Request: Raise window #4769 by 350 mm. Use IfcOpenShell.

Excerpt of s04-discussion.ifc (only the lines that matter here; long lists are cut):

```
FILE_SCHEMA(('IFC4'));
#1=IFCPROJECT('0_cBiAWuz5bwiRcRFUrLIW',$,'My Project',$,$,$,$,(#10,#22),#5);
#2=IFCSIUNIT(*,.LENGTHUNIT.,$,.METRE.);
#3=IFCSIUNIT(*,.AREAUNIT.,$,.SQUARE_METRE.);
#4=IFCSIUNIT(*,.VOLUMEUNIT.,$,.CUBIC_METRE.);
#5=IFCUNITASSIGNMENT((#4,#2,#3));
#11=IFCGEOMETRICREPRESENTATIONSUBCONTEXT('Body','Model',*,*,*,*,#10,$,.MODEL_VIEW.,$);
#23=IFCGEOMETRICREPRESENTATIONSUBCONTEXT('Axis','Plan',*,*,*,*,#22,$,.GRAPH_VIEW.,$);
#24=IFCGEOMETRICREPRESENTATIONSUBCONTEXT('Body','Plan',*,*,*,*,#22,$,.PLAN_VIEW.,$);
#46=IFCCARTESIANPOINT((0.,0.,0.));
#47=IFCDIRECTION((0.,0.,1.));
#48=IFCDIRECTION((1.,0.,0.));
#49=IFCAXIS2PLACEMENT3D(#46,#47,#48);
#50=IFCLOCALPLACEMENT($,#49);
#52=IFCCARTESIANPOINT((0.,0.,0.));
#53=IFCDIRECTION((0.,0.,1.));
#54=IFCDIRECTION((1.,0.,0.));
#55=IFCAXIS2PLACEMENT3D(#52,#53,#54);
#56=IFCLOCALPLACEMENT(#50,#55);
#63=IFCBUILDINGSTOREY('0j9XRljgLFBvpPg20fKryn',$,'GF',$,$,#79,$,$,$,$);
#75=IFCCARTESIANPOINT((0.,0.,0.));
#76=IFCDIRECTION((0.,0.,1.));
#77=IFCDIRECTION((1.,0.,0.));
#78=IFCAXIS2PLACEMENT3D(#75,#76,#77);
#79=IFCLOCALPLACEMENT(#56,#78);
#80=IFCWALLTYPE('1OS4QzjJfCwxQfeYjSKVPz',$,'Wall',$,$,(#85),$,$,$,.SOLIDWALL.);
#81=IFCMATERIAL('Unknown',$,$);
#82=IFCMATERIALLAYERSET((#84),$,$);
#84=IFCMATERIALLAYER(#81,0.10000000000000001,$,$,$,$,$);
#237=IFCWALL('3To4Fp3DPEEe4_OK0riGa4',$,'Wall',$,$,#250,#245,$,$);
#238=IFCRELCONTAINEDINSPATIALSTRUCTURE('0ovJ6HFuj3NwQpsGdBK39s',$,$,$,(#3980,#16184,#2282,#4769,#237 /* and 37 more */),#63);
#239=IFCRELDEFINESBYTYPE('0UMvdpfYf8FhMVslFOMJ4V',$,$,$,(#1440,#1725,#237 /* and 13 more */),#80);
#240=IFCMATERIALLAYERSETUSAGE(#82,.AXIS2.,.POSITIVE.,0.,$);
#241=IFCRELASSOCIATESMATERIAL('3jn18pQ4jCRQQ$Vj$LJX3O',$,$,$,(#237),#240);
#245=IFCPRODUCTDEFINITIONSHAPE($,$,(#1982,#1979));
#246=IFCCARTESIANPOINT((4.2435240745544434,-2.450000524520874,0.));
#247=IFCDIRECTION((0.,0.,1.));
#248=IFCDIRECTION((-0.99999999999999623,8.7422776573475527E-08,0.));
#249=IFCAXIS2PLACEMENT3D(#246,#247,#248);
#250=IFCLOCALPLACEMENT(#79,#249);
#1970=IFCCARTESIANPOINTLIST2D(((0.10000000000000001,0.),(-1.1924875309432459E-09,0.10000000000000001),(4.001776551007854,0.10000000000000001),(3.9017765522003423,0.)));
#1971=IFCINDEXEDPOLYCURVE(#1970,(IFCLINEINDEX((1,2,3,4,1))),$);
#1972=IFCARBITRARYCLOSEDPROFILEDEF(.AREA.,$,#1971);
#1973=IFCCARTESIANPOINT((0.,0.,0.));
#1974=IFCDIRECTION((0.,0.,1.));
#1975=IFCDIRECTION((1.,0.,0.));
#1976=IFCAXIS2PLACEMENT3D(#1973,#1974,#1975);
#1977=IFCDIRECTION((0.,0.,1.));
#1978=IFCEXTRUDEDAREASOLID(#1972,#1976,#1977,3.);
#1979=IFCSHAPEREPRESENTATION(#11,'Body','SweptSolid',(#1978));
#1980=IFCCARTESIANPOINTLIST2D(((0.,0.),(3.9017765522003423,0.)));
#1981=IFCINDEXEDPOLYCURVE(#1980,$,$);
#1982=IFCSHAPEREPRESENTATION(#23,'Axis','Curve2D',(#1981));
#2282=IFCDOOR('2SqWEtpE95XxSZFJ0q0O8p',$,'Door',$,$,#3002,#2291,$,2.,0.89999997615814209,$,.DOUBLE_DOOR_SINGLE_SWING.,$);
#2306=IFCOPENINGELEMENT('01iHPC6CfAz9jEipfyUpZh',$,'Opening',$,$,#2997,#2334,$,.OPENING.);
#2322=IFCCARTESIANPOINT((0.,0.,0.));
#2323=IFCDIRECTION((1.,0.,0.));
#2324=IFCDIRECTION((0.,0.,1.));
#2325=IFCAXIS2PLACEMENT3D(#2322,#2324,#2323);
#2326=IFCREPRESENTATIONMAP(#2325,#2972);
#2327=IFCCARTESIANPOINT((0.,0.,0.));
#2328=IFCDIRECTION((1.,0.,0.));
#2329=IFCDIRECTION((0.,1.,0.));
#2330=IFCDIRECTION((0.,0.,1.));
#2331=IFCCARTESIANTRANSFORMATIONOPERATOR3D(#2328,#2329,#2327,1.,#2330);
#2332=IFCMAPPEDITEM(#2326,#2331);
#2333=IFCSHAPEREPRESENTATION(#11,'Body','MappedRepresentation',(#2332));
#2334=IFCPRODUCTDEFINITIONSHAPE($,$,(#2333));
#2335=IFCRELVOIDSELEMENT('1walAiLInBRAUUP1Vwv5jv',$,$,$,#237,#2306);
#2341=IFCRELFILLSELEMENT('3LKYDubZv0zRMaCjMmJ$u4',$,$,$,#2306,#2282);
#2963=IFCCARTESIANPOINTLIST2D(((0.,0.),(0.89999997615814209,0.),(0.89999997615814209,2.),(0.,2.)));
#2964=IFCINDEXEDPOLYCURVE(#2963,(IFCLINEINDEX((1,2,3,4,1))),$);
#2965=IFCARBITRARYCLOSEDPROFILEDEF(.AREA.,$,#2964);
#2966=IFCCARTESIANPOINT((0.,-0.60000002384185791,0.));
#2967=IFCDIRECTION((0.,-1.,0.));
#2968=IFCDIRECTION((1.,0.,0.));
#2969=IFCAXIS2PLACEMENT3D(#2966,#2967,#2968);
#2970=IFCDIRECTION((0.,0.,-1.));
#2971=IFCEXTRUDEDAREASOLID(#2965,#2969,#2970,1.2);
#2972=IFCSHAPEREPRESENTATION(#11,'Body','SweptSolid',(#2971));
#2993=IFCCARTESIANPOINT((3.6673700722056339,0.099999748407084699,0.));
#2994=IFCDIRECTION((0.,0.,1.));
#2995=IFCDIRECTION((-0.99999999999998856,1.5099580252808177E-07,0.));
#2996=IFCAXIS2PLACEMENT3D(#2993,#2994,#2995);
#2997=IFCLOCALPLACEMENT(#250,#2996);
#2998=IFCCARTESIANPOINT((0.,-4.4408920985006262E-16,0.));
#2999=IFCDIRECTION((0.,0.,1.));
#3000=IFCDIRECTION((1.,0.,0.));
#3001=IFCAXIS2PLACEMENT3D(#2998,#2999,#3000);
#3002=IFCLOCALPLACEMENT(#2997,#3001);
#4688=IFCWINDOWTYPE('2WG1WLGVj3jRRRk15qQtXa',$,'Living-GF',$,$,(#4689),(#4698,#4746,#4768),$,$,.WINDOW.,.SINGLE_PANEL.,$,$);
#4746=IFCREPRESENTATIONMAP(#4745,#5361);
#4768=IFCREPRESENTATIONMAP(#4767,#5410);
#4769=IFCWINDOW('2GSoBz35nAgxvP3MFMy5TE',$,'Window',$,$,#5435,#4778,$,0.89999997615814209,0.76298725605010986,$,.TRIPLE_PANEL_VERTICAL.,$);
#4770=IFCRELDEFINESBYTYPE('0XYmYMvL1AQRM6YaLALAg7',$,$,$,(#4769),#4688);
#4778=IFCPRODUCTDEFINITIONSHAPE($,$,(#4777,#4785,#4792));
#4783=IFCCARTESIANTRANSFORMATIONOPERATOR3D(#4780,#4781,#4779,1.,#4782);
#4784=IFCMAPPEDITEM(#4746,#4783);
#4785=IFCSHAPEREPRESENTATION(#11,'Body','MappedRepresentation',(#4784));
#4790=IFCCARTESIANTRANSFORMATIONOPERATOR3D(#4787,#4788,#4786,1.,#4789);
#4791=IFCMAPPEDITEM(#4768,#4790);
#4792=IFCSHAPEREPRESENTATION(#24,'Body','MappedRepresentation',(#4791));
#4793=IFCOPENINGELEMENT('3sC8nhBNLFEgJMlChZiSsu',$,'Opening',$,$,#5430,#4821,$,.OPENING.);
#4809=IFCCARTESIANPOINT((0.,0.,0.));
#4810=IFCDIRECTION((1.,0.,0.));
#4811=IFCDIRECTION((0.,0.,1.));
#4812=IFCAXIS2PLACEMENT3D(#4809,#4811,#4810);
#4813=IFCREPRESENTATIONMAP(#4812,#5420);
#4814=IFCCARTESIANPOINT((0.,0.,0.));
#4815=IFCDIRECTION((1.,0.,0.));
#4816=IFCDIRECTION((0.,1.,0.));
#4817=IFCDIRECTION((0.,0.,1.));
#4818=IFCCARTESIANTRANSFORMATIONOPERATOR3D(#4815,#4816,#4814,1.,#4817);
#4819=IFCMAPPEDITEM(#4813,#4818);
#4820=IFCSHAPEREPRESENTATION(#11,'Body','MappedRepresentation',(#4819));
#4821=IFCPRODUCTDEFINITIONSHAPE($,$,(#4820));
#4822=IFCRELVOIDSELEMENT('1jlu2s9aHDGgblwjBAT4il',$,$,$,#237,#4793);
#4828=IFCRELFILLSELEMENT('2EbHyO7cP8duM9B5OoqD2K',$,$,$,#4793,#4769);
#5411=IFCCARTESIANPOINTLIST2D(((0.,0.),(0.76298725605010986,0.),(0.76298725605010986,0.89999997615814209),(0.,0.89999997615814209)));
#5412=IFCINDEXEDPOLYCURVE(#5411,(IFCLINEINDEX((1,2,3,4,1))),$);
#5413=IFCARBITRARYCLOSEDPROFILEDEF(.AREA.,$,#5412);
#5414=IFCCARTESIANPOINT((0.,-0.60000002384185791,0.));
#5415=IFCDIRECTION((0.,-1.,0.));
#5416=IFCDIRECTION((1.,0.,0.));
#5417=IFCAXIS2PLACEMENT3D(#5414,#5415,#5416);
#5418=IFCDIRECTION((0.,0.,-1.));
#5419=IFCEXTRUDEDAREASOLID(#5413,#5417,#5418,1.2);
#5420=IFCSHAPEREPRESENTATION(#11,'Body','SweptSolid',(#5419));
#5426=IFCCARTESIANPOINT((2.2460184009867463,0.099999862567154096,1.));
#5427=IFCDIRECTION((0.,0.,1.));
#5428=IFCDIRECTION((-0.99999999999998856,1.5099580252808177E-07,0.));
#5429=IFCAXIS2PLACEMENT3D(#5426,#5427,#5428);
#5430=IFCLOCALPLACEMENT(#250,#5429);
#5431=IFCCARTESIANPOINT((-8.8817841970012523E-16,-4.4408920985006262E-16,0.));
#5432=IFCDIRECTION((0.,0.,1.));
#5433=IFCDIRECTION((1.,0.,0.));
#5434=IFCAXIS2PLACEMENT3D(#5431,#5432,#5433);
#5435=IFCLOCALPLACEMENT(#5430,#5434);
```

```python
import numpy as np
import ifcopenshell
import ifcopenshell.api.geometry
import ifcopenshell.util.placement
import ifcopenshell.util.unit

model = ifcopenshell.open("s04-discussion.ifc")
unit_scale = ifcopenshell.util.unit.calculate_unit_scale(model)

window = model.by_id(4769)
opening = window.FillsVoids[0].RelatingOpeningElement
dz = 0.35 / unit_scale

shift = np.array([0.0, 0.0, dz])
# The window is placed relative to its opening, so it follows when the opening moves.
matrix = ifcopenshell.util.placement.get_local_placement(opening.ObjectPlacement)
matrix[:3, 3] += shift
ifcopenshell.api.geometry.edit_object_placement(
    model, product=opening, matrix=matrix, is_si=False, should_transform_children=True
)

print(f"moved by {dz * unit_scale:+.3f} m")

model.write("s04-discussion_updated.ifc")
```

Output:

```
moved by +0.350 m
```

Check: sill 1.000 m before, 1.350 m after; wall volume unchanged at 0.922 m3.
